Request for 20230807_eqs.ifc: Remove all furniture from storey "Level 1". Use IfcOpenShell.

First a look at what the model holds.

```python
import ifcopenshell
import ifcopenshell.util.element

model = ifcopenshell.open("20230807_eqs.ifc")
print(model.schema)
storey = next(s for s in model.by_type("IfcBuildingStorey") if s.Name == "Level 1")
furniture = [e for e in ifcopenshell.util.element.get_decomposition(storey) if e.is_a("IfcFurnishingElement")]
seen = {}
for e in furniture:
    element_type = ifcopenshell.util.element.get_type(e)
    name = element_type.Name if element_type not in (None, e) else None
    seen[name] = seen.get(name, 0) + 1
for name, count in sorted(seen.items(), key=str):
    print(count, "x", name)
```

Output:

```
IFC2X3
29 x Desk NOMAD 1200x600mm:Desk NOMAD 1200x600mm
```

```python
import ifcopenshell
import ifcopenshell.api.root
import ifcopenshell.util.element

model = ifcopenshell.open("20230807_eqs.ifc")

storey = next(s for s in model.by_type("IfcBuildingStorey") if s.Name == "Level 1")
furniture = [e for e in ifcopenshell.util.element.get_decomposition(storey) if e.is_a("IfcFurnishingElement")]

for e in furniture:
    ifcopenshell.api.root.remove_product(model, product=e)
print(len(furniture), "removed")

model.write("20230807_eqs_v2.ifc")
```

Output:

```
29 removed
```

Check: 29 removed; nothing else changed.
